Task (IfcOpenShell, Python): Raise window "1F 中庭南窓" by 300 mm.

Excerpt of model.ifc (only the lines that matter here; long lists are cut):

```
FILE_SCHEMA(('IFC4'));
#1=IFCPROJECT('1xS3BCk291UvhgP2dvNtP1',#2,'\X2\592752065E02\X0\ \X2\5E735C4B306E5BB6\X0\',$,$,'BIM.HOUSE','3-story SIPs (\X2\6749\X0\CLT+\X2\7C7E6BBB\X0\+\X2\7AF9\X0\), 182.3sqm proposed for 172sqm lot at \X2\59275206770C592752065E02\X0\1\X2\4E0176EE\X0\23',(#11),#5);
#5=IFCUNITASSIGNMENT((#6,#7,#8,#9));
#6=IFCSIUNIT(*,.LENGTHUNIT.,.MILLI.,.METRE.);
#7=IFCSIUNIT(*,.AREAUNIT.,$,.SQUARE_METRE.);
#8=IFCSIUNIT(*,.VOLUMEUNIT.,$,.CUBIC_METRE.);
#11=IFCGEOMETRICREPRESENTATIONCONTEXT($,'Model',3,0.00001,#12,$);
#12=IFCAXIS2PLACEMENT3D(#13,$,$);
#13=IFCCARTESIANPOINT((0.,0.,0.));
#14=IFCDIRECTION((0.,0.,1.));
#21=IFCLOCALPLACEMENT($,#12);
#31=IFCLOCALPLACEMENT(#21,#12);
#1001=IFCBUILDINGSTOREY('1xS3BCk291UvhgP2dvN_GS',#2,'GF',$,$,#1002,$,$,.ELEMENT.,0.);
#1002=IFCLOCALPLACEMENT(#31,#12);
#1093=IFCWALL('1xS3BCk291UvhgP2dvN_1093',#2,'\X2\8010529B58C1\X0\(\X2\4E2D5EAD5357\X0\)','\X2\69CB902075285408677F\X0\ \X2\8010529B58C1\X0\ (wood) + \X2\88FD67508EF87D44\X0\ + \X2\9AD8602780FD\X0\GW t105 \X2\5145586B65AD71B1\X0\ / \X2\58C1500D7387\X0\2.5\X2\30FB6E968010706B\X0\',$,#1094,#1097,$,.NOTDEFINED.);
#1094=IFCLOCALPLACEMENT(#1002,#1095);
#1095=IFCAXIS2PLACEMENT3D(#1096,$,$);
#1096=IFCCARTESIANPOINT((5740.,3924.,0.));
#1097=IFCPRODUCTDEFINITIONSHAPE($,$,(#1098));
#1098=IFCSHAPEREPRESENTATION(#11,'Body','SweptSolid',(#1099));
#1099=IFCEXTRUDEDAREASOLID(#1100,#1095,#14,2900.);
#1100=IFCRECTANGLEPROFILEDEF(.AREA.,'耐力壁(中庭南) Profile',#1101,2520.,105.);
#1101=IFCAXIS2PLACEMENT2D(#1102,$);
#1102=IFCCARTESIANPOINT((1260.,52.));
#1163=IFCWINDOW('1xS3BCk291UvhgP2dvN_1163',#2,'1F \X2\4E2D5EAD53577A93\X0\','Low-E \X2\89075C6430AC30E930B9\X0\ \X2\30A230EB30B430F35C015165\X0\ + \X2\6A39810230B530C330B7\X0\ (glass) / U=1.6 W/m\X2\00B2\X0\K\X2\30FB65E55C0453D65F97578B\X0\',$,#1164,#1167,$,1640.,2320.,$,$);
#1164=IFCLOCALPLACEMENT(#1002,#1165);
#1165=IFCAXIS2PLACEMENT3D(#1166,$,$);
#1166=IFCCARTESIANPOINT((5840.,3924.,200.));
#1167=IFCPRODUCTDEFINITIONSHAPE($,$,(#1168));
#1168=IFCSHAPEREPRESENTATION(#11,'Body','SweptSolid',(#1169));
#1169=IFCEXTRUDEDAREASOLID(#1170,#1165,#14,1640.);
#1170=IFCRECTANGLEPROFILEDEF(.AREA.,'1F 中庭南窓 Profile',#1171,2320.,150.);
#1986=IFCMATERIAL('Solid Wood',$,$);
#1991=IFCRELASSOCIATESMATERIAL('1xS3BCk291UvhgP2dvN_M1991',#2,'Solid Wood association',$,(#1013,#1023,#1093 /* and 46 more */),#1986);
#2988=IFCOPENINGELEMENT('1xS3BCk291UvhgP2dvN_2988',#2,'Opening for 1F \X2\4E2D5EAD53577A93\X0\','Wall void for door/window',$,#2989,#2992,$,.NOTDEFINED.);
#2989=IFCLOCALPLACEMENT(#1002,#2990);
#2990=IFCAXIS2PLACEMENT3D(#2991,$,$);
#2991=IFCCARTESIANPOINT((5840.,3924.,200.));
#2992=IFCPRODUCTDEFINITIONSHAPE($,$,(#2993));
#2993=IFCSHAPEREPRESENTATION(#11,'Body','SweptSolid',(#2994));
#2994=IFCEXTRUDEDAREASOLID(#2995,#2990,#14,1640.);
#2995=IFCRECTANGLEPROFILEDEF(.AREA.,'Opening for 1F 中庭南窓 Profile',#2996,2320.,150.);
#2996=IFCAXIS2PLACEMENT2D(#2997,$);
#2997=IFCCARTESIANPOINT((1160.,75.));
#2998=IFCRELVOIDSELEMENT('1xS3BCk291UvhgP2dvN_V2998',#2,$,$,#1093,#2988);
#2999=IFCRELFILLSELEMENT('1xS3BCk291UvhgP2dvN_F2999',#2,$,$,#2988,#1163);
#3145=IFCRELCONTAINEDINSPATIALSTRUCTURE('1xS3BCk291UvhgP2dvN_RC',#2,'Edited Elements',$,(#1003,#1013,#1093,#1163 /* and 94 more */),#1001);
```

```python
import numpy as np
import ifcopenshell
import ifcopenshell.api.geometry
import ifcopenshell.util.placement
import ifcopenshell.util.unit

model = ifcopenshell.open("model.ifc")
unit_scale = ifcopenshell.util.unit.calculate_unit_scale(model)

window = model.by_guid("1xS3BCk291UvhgP2dvN_1163")
opening = window.FillsVoids[0].RelatingOpeningElement
dz = 0.3 / unit_scale

shift = np.array([0.0, 0.0, dz])
# The window is not placed relative to its opening, so move both.
for product in (opening, window):
    matrix = ifcopenshell.util.placement.get_local_placement(product.ObjectPlacement)
    matrix[:3, 3] += shift
    ifcopenshell.api.geometry.edit_object_placement(model, product=product, matrix=matrix, is_si=False)

print(f"moved by {dz * unit_scale:+.3f} m")

model.write("model_updated.ifc")
```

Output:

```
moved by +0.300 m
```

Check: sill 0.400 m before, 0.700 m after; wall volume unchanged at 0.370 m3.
